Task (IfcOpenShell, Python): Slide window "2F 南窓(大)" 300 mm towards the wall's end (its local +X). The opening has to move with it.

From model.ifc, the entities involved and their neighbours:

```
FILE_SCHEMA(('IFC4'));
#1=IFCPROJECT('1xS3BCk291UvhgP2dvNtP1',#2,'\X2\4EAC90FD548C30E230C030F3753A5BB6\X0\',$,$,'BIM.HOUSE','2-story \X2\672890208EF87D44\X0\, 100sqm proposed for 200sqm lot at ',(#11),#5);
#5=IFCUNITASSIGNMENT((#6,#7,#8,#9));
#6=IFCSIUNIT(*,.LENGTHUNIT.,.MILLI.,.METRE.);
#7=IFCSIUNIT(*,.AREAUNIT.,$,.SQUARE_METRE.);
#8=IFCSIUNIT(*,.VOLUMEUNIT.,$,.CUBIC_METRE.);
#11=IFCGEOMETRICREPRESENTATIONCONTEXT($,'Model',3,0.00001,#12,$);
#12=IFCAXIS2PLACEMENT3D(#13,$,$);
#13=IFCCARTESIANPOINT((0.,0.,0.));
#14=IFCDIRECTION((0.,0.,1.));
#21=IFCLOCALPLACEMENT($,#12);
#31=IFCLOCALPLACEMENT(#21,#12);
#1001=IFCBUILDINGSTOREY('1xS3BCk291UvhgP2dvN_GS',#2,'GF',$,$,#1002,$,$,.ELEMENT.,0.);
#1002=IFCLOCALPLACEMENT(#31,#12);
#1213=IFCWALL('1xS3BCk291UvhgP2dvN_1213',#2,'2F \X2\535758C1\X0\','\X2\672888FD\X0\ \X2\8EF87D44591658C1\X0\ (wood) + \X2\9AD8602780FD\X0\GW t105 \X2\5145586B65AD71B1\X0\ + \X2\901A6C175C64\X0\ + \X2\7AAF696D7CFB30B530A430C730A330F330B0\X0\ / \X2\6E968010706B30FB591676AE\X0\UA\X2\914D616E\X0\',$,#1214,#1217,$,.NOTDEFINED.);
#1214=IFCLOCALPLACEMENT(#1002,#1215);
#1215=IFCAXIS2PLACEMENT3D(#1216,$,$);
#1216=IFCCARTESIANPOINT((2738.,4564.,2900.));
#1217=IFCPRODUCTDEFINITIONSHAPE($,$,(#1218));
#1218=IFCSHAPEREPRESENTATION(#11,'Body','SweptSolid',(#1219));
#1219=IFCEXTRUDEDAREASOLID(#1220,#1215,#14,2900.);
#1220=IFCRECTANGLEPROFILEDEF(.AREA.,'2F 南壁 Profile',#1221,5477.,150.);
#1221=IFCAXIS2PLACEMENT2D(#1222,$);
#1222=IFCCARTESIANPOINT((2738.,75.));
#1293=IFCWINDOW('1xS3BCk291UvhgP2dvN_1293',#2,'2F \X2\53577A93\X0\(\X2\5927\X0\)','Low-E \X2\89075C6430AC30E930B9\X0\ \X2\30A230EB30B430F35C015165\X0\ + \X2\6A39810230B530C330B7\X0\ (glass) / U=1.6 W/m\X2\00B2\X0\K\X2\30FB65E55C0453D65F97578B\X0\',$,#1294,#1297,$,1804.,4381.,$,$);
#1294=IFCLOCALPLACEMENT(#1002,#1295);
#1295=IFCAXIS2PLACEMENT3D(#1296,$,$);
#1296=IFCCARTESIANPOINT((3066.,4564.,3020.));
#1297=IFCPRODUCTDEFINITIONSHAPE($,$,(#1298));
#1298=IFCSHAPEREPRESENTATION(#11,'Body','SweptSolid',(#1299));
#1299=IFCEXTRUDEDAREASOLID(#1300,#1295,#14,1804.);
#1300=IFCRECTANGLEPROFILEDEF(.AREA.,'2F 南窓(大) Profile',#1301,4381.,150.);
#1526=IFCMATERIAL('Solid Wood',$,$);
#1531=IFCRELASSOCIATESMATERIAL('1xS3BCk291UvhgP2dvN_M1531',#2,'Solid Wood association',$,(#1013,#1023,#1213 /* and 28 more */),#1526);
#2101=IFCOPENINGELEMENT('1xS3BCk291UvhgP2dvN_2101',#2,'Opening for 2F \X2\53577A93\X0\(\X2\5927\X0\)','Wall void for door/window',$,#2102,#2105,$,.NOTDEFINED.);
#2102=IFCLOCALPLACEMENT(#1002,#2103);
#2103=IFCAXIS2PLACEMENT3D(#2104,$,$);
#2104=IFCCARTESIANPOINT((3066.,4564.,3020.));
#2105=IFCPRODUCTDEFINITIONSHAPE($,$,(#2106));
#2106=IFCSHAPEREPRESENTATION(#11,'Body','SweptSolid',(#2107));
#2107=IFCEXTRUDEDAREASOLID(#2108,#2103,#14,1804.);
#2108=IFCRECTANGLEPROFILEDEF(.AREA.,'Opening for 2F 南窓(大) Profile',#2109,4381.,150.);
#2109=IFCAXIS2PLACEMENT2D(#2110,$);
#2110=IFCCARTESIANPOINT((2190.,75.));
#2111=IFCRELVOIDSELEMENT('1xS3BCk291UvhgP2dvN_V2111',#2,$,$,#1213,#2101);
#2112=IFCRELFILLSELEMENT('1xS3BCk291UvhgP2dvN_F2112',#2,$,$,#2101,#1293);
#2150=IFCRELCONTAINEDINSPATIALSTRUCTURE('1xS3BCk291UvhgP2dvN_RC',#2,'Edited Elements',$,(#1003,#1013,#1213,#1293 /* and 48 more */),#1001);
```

```python
import ifcopenshell
import ifcopenshell.api.geometry
import ifcopenshell.util.placement
import ifcopenshell.util.unit

model = ifcopenshell.open("model.ifc")
unit_scale = ifcopenshell.util.unit.calculate_unit_scale(model)

window = model.by_guid("1xS3BCk291UvhgP2dvN_1293")
opening = window.FillsVoids[0].RelatingOpeningElement
wall = opening.VoidsElements[0].RelatingBuildingElement

wall_matrix = ifcopenshell.util.placement.get_local_placement(wall.ObjectPlacement)
shift = wall_matrix[:3, 0] * 0.3 / unit_scale
before = ifcopenshell.util.placement.get_local_placement(window.ObjectPlacement)[:3, 3].copy()

# The window is not placed relative to its opening, so move both.
for product in (opening, window):
    matrix = ifcopenshell.util.placement.get_local_placement(product.ObjectPlacement)
    matrix[:3, 3] += shift
    ifcopenshell.api.geometry.edit_object_placement(model, product=product, matrix=matrix, is_si=False)

after = ifcopenshell.util.placement.get_local_placement(window.ObjectPlacement)[:3, 3]
print("window moved by", (after - before).round(3) + 0.0)

model.write("model_v2.ifc")
```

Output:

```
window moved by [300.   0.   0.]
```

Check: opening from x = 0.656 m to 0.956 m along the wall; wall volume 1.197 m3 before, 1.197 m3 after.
